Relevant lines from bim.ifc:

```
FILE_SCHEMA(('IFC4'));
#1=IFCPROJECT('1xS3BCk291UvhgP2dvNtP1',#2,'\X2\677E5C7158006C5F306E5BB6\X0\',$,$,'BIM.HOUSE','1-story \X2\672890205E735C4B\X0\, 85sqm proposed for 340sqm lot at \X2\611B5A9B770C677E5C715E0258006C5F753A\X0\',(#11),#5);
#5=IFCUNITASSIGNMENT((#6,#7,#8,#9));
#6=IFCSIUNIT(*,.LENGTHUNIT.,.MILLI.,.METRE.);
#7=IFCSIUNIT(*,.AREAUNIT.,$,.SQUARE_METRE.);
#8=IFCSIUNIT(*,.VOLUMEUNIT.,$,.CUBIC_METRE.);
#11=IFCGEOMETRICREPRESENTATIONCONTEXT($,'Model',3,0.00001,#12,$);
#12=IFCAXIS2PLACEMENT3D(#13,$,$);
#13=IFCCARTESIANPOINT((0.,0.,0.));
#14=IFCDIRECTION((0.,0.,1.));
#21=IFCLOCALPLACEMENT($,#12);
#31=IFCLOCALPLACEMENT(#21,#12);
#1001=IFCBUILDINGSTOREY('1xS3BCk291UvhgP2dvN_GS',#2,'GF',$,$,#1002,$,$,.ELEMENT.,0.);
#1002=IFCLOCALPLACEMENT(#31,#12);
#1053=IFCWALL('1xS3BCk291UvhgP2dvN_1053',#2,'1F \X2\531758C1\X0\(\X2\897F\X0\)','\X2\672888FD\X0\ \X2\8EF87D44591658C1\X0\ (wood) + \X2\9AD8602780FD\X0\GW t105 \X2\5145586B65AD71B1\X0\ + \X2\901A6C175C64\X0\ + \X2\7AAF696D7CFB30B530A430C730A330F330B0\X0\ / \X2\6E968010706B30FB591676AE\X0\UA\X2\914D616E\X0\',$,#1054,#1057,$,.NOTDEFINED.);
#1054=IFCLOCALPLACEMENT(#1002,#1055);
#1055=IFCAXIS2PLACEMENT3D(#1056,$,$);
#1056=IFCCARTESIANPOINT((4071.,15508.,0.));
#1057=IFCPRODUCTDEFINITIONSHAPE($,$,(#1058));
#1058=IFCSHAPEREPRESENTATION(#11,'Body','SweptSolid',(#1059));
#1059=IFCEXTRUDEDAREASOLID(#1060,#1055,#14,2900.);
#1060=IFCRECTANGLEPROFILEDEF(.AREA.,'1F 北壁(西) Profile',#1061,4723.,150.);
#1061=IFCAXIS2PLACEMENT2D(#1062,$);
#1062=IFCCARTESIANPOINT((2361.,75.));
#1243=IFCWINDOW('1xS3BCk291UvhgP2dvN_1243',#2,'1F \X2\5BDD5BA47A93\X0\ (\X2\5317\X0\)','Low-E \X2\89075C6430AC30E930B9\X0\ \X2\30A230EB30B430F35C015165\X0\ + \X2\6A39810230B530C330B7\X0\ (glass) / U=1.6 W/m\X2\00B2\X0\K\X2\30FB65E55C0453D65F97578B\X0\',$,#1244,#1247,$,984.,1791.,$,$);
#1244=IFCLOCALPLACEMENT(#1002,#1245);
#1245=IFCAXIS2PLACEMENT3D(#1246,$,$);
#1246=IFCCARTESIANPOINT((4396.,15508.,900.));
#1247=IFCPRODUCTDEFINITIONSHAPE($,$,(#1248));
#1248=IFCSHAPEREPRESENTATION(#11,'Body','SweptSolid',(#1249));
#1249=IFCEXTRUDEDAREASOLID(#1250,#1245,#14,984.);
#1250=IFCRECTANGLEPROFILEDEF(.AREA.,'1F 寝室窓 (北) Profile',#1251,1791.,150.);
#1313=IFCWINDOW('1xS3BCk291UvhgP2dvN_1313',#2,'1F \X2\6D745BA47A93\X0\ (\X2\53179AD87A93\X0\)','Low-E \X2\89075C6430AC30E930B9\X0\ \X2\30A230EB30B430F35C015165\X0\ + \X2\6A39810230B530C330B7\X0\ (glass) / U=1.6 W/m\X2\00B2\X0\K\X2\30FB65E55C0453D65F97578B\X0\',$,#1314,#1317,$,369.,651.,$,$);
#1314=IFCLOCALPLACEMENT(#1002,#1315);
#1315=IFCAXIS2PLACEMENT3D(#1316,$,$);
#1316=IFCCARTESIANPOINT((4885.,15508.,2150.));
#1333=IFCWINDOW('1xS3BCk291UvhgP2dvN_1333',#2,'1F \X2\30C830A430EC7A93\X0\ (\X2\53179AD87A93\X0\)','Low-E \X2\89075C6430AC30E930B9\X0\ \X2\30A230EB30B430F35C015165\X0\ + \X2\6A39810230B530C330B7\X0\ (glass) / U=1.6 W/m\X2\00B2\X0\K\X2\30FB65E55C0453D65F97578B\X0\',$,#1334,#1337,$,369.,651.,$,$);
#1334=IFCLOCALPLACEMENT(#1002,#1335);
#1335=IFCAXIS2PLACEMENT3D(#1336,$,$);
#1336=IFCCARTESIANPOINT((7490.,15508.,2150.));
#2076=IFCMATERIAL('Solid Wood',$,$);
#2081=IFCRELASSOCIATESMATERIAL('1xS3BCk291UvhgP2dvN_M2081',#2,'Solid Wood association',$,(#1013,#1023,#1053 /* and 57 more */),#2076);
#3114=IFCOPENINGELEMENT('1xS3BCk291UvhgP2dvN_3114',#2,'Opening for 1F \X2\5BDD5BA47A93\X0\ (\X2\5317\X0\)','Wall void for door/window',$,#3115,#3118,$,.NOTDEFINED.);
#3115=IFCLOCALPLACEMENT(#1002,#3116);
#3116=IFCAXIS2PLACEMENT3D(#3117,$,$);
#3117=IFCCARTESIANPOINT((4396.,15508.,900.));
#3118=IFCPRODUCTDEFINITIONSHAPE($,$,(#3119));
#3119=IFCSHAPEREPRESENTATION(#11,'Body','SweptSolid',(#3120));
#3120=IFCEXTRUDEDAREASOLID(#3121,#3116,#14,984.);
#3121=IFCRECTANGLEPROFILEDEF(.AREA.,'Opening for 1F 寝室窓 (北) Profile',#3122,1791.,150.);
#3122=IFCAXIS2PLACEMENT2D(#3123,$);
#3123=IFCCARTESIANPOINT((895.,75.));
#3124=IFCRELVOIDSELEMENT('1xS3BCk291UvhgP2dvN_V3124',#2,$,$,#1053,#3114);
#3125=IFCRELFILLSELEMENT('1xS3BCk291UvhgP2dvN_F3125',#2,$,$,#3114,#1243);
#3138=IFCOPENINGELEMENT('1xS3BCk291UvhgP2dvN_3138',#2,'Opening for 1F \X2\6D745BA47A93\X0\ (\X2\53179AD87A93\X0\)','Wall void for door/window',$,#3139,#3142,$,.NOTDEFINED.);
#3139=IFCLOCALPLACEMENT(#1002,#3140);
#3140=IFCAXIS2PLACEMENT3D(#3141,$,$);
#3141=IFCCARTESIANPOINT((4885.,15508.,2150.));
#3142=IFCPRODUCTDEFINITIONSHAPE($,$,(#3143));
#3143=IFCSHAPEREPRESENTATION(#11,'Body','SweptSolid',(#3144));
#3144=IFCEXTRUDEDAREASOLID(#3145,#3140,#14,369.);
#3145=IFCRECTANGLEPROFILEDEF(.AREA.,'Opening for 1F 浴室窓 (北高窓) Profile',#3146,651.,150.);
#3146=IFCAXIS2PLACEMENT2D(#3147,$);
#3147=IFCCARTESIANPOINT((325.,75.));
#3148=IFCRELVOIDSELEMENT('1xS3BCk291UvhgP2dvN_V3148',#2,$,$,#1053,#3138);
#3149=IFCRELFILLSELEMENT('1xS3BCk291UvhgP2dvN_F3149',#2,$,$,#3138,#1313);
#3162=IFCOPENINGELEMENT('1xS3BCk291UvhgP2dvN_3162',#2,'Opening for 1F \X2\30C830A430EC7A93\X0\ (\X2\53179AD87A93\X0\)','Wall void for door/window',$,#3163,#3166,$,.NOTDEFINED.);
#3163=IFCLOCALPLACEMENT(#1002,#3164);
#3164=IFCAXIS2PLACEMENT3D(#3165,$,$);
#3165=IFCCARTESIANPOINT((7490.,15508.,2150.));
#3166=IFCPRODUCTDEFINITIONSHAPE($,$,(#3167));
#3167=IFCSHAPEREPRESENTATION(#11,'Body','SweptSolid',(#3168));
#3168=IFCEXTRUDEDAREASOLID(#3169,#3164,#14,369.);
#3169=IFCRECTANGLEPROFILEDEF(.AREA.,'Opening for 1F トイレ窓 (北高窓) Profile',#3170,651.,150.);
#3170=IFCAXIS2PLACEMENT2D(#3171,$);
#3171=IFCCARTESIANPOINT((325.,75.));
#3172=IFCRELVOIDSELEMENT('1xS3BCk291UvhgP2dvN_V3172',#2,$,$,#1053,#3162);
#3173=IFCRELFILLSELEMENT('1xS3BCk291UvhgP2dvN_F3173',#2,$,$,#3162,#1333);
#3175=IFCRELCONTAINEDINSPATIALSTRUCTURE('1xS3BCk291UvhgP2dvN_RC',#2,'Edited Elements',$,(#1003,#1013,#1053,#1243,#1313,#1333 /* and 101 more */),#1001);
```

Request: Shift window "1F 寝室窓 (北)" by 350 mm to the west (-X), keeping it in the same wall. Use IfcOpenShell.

```python
import ifcopenshell
import ifcopenshell.api.geometry
import ifcopenshell.util.placement
import ifcopenshell.util.unit

model = ifcopenshell.open("bim.ifc")
unit_scale = ifcopenshell.util.unit.calculate_unit_scale(model)

window = model.by_guid("1xS3BCk291UvhgP2dvN_1243")
opening = window.FillsVoids[0].RelatingOpeningElement
wall = opening.VoidsElements[0].RelatingBuildingElement

wall_matrix = ifcopenshell.util.placement.get_local_placement(wall.ObjectPlacement)
shift = wall_matrix[:3, 0] * -0.35 / unit_scale
before = ifcopenshell.util.placement.get_local_placement(window.ObjectPlacement)[:3, 3].copy()

# The window is not placed relative to its opening, so move both.
for product in (opening, window):
    matrix = ifcopenshell.util.placement.get_local_placement(product.ObjectPlacement)
    matrix[:3, 3] += shift
    ifcopenshell.api.geometry.edit_object_placement(model, product=product, matrix=matrix, is_si=False)

after = ifcopenshell.util.placement.get_local_placement(window.ObjectPlacement)[:3, 3]
print("window moved by", (after - before).round(3) + 0.0)

model.write("bim_updated.ifc")
```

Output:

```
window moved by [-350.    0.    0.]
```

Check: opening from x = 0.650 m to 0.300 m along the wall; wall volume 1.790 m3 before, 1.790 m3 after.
